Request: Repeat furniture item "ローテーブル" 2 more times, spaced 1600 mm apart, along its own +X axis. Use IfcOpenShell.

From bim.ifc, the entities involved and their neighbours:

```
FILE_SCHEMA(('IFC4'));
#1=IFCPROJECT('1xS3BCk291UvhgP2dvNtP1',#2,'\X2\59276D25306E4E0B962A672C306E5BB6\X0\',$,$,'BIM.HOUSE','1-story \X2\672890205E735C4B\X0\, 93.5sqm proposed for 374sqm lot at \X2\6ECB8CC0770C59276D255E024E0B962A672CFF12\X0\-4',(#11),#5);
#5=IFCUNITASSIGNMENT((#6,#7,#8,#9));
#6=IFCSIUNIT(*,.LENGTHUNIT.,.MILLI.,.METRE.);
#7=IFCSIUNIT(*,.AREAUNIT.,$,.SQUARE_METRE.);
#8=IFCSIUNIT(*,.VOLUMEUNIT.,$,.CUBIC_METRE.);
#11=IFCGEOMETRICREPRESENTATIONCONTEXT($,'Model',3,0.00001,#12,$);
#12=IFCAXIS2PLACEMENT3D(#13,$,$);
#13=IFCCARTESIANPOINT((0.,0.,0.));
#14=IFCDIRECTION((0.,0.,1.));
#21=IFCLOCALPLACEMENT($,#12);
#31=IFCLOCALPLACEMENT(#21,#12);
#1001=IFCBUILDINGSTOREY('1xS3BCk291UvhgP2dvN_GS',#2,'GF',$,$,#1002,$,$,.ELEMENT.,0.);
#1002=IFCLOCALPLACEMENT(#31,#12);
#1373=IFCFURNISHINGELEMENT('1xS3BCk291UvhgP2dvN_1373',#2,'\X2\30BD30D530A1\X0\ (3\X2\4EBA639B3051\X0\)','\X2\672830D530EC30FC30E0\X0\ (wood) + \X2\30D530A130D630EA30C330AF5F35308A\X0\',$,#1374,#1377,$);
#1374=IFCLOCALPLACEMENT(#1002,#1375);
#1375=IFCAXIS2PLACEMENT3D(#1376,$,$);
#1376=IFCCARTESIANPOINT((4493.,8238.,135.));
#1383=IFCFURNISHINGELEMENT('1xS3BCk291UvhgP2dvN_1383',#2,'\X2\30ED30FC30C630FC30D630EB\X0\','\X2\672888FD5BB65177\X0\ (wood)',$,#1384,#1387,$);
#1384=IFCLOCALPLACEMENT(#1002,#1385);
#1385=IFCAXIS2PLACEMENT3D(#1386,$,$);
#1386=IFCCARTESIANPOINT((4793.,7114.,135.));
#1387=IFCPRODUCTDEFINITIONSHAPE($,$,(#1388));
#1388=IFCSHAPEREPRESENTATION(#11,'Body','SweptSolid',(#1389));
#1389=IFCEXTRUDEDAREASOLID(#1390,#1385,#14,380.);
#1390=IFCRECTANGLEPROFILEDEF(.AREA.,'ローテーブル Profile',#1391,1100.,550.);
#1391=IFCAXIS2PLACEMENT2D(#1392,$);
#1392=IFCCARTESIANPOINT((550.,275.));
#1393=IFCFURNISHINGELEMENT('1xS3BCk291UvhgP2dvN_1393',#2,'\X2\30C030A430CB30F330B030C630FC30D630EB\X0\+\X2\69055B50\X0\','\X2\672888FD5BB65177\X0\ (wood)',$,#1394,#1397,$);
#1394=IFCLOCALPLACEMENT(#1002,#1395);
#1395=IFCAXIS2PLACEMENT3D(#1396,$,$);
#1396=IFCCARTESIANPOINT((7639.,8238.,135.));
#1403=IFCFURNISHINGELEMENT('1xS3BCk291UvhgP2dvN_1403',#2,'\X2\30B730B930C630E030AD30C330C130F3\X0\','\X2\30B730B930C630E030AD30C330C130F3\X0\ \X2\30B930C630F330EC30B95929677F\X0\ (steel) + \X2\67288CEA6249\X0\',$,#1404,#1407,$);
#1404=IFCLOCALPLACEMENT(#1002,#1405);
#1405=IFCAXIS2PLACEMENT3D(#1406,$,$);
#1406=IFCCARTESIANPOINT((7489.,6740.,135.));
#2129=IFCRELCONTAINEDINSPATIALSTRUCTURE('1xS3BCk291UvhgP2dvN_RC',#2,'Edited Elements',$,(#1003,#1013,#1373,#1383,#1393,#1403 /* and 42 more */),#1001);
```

```python
import ifcopenshell
import ifcopenshell.api.geometry
import ifcopenshell.api.root
import ifcopenshell.util.element
import ifcopenshell.util.placement
import ifcopenshell.util.unit

model = ifcopenshell.open("bim.ifc")
unit_scale = ifcopenshell.util.unit.calculate_unit_scale(model)


def reuse_history(source, copy):
    """copy_class also copies each property set's owner history, people and application; keep the originals."""
    for rel in copy.IsDefinedBy:
        if rel.is_a("IfcRelDefinesByProperties") and (history := rel.RelatingPropertyDefinition.OwnerHistory):
            rel.RelatingPropertyDefinition.OwnerHistory = source.OwnerHistory
            ifcopenshell.util.element.remove_deep2(model, history)


source = model.by_guid("1xS3BCk291UvhgP2dvN_1383")
base = ifcopenshell.util.placement.get_local_placement(source.ObjectPlacement)
step = base[:3, 0] * 1.6 / unit_scale

for i in range(1, 3):
    copy = ifcopenshell.api.root.copy_class(model, product=source)
    copy.Representation = ifcopenshell.util.element.copy_deep(
        model, source.Representation, exclude=["IfcGeometricRepresentationContext", "IfcRepresentationMap"]
    )
    reuse_history(source, copy)
    matrix = base.copy()
    matrix[:3, 3] += i * step
    print("added at", matrix[:3, 3].round(3) + 0.0)
    ifcopenshell.api.geometry.edit_object_placement(model, product=copy, matrix=matrix, is_si=False)

model.write("bim_updated.ifc")
```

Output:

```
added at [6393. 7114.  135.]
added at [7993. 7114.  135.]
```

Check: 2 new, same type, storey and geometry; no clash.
